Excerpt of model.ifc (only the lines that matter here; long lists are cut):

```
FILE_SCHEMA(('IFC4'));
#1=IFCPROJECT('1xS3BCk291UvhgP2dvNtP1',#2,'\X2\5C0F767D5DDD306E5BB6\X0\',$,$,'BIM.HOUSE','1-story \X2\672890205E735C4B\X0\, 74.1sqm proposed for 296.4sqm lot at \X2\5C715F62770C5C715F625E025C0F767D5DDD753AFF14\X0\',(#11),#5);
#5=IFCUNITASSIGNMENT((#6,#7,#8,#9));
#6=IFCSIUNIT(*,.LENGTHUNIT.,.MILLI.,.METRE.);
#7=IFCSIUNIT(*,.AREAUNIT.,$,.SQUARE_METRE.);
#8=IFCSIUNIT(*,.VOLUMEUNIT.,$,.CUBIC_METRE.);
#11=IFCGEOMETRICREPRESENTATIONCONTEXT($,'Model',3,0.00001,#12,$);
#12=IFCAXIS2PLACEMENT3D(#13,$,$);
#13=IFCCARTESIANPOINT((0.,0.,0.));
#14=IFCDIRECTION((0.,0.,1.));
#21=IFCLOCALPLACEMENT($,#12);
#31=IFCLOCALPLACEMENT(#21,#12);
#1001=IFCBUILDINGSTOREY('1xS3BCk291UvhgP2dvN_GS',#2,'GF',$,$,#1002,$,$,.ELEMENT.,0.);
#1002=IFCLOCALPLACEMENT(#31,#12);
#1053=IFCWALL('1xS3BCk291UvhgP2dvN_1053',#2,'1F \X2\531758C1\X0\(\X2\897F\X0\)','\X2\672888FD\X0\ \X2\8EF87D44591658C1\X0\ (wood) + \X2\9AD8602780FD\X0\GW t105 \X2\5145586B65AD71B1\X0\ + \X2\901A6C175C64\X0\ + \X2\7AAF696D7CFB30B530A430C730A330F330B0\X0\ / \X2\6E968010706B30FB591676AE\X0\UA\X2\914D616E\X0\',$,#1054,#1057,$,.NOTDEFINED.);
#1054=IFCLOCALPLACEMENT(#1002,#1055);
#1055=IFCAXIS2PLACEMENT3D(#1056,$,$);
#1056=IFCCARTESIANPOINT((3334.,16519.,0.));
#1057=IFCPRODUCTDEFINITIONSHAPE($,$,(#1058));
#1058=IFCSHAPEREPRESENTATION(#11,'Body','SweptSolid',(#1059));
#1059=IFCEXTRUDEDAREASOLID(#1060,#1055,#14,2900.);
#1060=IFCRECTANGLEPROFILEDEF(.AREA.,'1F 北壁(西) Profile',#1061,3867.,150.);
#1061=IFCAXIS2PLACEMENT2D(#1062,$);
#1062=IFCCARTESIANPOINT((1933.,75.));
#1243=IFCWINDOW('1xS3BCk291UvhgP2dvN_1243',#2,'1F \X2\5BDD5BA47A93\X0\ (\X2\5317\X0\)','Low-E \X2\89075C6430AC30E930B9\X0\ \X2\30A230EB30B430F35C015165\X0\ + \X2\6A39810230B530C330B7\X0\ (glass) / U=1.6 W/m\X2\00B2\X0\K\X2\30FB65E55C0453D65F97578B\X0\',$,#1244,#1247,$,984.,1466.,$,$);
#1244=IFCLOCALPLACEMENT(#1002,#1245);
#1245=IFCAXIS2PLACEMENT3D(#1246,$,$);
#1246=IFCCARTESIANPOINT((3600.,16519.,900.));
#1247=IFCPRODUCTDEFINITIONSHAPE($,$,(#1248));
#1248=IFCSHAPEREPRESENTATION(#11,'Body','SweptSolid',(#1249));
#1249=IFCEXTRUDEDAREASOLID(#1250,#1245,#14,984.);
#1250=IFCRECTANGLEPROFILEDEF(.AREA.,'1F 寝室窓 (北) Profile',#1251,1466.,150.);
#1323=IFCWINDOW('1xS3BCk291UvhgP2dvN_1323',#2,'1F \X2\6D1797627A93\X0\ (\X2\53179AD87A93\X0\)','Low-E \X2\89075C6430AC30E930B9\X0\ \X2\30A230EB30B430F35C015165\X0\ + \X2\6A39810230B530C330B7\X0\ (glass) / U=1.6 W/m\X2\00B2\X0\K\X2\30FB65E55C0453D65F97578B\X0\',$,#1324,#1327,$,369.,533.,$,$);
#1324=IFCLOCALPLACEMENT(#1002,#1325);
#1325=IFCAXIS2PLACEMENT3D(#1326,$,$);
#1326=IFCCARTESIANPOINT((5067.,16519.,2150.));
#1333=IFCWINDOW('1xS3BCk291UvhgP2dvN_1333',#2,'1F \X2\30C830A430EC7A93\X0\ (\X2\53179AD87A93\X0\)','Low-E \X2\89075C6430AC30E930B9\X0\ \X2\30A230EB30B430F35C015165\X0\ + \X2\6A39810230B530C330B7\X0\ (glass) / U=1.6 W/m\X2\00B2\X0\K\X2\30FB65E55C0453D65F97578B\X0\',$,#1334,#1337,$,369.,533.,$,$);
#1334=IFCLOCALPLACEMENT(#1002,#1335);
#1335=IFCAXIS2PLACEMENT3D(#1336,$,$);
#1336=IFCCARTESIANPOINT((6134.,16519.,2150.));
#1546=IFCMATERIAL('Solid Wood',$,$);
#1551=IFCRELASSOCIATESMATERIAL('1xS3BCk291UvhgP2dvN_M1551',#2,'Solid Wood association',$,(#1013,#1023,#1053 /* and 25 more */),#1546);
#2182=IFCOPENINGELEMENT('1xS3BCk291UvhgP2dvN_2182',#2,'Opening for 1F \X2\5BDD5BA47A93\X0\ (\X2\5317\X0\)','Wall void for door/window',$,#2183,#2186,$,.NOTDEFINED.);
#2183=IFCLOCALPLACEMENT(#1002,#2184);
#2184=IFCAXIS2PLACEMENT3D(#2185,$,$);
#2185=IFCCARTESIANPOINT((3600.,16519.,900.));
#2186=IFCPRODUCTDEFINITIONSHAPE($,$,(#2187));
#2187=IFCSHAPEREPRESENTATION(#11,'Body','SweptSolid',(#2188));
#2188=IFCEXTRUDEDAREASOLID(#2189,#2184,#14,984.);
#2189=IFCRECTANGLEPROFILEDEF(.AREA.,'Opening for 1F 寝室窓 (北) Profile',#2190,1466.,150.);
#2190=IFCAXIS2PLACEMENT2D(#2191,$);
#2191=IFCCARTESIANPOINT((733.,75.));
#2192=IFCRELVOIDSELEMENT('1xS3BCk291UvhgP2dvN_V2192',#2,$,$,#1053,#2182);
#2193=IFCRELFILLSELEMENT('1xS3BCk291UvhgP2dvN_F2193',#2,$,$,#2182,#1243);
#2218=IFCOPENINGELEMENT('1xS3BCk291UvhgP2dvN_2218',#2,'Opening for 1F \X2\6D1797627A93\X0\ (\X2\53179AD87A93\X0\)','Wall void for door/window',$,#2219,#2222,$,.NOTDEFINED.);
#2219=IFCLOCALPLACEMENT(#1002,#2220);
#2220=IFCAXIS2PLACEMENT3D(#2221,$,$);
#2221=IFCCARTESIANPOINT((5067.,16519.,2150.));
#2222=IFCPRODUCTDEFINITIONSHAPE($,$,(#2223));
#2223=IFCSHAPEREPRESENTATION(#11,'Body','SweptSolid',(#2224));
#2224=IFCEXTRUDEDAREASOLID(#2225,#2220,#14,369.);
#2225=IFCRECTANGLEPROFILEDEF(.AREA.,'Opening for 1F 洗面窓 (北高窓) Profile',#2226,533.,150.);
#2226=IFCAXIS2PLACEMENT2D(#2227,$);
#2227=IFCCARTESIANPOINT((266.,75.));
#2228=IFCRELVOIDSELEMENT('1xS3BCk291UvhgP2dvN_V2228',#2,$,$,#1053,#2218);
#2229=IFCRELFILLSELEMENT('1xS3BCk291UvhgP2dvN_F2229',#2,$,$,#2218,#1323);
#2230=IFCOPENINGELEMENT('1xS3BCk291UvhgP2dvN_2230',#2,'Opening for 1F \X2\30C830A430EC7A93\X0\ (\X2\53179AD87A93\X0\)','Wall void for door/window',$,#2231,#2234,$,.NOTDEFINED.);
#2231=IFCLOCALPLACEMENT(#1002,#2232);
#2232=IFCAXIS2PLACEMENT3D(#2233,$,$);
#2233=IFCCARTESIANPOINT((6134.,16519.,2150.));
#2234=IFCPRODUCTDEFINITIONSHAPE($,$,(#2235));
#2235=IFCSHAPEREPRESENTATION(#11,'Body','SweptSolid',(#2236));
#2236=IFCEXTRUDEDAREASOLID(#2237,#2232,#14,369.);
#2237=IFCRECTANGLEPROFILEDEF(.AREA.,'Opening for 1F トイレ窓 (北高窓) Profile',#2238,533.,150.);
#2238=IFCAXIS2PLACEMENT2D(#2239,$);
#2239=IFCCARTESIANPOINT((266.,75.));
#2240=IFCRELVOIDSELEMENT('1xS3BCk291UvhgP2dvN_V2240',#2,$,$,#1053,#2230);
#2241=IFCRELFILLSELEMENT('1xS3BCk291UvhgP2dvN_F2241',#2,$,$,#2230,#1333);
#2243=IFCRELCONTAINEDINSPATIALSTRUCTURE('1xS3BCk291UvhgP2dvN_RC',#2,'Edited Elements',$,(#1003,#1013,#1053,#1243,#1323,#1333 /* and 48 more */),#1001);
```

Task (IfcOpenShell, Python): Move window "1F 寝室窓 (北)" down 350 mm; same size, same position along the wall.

```python
import numpy as np
import ifcopenshell
import ifcopenshell.api.geometry
import ifcopenshell.util.placement
import ifcopenshell.util.unit

model = ifcopenshell.open("model.ifc")
unit_scale = ifcopenshell.util.unit.calculate_unit_scale(model)

window = model.by_guid("1xS3BCk291UvhgP2dvN_1243")
opening = window.FillsVoids[0].RelatingOpeningElement
dz = -0.35 / unit_scale

shift = np.array([0.0, 0.0, dz])
# The window is not placed relative to its opening, so move both.
for product in (opening, window):
    matrix = ifcopenshell.util.placement.get_local_placement(product.ObjectPlacement)
    matrix[:3, 3] += shift
    ifcopenshell.api.geometry.edit_object_placement(model, product=product, matrix=matrix, is_si=False)

print(f"moved by {dz * unit_scale:+.3f} m")

model.write("model-out.ifc")
```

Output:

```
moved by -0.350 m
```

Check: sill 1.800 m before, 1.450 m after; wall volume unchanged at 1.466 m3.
